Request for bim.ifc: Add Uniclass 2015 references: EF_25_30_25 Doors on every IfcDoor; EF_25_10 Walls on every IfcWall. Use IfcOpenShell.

First a look at what the model holds.

```python
import ifcopenshell

model = ifcopenshell.open("bim.ifc")
print(model.schema)
print("classifications:", [c.Name for c in model.by_type("IfcClassification")])
for ifc_class in ("IfcDoor", "IfcRoof", "IfcStair", "IfcWall", "IfcWindow"):
    print(ifc_class, len(model.by_type(ifc_class)))
```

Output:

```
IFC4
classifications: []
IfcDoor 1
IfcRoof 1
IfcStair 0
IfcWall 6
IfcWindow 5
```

```python
import ifcopenshell
import ifcopenshell.api.classification

model = ifcopenshell.open("bim.ifc")

system = ifcopenshell.api.classification.add_classification(model, classification="Uniclass 2015")

codes = {
    "IfcDoor": ("EF_25_30_25", "Doors"),
    "IfcWall": ("EF_25_10", "Walls"),
}
for ifc_class, (code, name) in codes.items():
    products = model.by_type(ifc_class)
    ifcopenshell.api.classification.add_reference(
        model, products=products, classification=system, identification=code, name=name
    )
    print(code, len(products))

model.write("bim_v2.ifc")
```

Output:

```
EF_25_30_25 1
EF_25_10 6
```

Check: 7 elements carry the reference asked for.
